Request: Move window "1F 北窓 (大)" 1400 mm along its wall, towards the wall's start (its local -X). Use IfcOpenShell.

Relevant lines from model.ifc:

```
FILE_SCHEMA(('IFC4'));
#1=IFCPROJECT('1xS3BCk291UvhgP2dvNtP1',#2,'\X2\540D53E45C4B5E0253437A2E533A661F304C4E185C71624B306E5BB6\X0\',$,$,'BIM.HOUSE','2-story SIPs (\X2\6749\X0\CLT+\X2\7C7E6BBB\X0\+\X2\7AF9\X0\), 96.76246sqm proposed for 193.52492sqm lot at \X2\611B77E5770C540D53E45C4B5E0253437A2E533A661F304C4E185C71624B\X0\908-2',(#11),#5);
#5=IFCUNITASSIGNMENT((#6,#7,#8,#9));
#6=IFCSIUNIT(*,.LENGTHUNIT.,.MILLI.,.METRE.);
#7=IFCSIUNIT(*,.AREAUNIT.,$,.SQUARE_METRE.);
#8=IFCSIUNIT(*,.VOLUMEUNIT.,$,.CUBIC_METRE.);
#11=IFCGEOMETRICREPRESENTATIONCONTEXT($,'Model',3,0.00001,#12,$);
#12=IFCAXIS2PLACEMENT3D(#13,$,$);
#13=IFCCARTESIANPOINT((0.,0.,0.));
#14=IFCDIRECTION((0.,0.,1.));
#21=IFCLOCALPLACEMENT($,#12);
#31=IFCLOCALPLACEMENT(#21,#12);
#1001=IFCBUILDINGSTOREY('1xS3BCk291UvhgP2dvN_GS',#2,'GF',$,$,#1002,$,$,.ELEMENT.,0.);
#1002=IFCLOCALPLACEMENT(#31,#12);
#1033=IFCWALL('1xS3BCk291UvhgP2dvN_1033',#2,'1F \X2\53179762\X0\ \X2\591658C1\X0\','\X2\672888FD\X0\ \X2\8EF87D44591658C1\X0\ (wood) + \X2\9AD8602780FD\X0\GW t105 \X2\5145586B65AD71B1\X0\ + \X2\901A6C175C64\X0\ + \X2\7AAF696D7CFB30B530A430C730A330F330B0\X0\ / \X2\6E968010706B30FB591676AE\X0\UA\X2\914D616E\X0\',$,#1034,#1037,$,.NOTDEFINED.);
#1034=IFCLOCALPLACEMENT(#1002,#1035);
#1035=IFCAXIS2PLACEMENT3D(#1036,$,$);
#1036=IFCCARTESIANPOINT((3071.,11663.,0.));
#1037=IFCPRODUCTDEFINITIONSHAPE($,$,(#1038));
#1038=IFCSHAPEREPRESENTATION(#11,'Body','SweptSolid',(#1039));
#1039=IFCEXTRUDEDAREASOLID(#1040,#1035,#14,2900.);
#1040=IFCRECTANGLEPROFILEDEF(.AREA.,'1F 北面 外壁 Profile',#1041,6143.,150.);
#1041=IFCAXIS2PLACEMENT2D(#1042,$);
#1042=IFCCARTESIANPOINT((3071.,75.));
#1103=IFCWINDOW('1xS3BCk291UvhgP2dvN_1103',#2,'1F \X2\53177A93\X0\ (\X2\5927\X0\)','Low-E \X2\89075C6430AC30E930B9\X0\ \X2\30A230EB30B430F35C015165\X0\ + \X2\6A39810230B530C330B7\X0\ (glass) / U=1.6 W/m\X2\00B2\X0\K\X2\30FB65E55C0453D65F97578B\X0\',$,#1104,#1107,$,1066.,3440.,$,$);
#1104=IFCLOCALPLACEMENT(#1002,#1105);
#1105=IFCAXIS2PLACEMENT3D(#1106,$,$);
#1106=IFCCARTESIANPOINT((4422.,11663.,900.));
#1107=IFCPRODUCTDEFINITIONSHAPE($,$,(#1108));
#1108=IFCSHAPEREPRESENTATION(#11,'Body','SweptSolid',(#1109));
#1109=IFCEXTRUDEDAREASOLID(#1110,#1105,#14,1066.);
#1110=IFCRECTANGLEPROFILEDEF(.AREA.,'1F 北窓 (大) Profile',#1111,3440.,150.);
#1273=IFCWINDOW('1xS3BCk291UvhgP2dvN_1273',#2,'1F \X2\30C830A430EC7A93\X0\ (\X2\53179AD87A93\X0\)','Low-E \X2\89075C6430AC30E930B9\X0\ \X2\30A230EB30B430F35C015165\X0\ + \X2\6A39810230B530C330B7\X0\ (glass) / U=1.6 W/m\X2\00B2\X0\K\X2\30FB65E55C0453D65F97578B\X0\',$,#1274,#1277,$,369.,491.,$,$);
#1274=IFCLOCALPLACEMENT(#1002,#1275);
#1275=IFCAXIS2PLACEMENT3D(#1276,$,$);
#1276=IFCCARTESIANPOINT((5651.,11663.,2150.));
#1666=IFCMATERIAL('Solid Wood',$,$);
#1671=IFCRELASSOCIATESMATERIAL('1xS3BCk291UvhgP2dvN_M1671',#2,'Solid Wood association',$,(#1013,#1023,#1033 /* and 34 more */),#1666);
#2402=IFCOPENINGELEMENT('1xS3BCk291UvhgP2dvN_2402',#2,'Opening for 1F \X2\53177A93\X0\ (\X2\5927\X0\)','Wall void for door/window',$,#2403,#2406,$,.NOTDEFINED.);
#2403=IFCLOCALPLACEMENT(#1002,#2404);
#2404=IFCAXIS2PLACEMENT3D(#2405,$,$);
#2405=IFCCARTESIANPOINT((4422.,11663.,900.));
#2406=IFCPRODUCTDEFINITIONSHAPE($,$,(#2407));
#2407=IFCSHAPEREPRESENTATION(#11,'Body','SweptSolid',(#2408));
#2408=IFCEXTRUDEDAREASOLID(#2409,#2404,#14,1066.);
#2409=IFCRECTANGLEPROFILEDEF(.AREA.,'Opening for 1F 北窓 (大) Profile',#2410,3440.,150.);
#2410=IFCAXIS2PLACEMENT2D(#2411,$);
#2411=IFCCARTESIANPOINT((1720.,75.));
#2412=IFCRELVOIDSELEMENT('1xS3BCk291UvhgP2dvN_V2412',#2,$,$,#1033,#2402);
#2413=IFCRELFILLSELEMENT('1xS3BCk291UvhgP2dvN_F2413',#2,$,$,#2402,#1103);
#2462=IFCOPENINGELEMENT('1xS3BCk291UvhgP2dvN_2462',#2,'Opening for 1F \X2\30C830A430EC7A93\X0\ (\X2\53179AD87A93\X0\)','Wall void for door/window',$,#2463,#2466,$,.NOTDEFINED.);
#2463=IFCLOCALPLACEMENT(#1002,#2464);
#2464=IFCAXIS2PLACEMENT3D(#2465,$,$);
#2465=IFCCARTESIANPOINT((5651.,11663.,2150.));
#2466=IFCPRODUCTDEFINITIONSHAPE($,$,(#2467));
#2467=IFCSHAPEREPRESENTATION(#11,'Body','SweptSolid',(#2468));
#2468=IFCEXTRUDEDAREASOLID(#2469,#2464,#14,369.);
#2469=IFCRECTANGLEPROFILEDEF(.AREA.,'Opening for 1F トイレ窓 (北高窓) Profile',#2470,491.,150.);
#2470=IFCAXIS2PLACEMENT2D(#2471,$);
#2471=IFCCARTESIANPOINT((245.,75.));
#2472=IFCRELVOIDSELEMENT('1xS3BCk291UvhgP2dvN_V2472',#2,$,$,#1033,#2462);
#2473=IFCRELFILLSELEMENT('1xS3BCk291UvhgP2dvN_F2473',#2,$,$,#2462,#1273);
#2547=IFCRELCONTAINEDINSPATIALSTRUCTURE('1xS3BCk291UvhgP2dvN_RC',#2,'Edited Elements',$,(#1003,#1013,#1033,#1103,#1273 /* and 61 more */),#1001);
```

```python
import ifcopenshell
import ifcopenshell.api.geometry
import ifcopenshell.util.placement
import ifcopenshell.util.unit

model = ifcopenshell.open("model.ifc")
unit_scale = ifcopenshell.util.unit.calculate_unit_scale(model)

window = model.by_guid("1xS3BCk291UvhgP2dvN_1103")
opening = window.FillsVoids[0].RelatingOpeningElement
wall = opening.VoidsElements[0].RelatingBuildingElement

wall_matrix = ifcopenshell.util.placement.get_local_placement(wall.ObjectPlacement)
shift = wall_matrix[:3, 0] * -1.4 / unit_scale
before = ifcopenshell.util.placement.get_local_placement(window.ObjectPlacement)[:3, 3].copy()

# The window is not placed relative to its opening, so move both.
for product in (opening, window):
    matrix = ifcopenshell.util.placement.get_local_placement(product.ObjectPlacement)
    matrix[:3, 3] += shift
    ifcopenshell.api.geometry.edit_object_placement(model, product=product, matrix=matrix, is_si=False)

after = ifcopenshell.util.placement.get_local_placement(window.ObjectPlacement)[:3, 3]
print("window moved by", (after - before).round(3) + 0.0)

model.write("model-out.ifc")
```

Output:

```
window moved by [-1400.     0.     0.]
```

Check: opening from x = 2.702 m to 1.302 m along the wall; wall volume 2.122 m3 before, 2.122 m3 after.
